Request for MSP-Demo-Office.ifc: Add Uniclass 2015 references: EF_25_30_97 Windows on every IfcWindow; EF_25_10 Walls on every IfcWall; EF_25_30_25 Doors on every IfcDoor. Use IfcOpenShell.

First a look at what the model holds.

```python
import ifcopenshell

model = ifcopenshell.open("MSP-Demo-Office.ifc")
print(model.schema)
print("classifications:", [c.Name for c in model.by_type("IfcClassification")])
for ifc_class in ("IfcDoor", "IfcRoof", "IfcStair", "IfcWall", "IfcWindow"):
    print(ifc_class, len(model.by_type(ifc_class)))
```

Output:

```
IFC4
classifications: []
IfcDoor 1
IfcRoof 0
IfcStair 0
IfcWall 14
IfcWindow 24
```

```python
import ifcopenshell
import ifcopenshell.api.classification

model = ifcopenshell.open("MSP-Demo-Office.ifc")

system = ifcopenshell.api.classification.add_classification(model, classification="Uniclass 2015")

codes = {
    "IfcWindow": ("EF_25_30_97", "Windows"),
    "IfcWall": ("EF_25_10", "Walls"),
    "IfcDoor": ("EF_25_30_25", "Doors"),
}
for ifc_class, (code, name) in codes.items():
    products = model.by_type(ifc_class)
    ifcopenshell.api.classification.add_reference(
        model, products=products, classification=system, identification=code, name=name
    )
    print(code, len(products))

model.write("MSP-Demo-Office_edited.ifc")
```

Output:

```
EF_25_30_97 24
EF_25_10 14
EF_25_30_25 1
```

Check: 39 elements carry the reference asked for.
